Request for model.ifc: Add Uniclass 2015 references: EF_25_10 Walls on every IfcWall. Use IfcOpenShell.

First a look at what the model holds.

```python
import ifcopenshell

model = ifcopenshell.open("model.ifc")
print(model.schema)
print("classifications:", [c.Name for c in model.by_type("IfcClassification")])
for ifc_class in ("IfcDoor", "IfcRoof", "IfcStair", "IfcWall", "IfcWindow"):
    print(ifc_class, len(model.by_type(ifc_class)))
```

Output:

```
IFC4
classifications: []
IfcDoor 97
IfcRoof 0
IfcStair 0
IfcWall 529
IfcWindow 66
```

```python
import ifcopenshell
import ifcopenshell.api.classification

model = ifcopenshell.open("model.ifc")

system = ifcopenshell.api.classification.add_classification(model, classification="Uniclass 2015")

codes = {
    "IfcWall": ("EF_25_10", "Walls"),
}
for ifc_class, (code, name) in codes.items():
    products = model.by_type(ifc_class)
    ifcopenshell.api.classification.add_reference(
        model, products=products, classification=system, identification=code, name=name
    )
    print(code, len(products))

model.write("model_rev.ifc")
```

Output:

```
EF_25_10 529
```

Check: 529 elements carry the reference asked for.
